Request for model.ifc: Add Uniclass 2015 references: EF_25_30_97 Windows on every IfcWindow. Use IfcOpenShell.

First a look at what the model holds.

```python
import ifcopenshell

model = ifcopenshell.open("model.ifc")
print(model.schema)
print("classifications:", [c.Name for c in model.by_type("IfcClassification")])
for ifc_class in ("IfcDoor", "IfcRoof", "IfcStair", "IfcWall", "IfcWindow"):
    print(ifc_class, len(model.by_type(ifc_class)))
```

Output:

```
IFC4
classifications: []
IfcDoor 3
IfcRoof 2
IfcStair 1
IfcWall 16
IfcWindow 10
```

```python
import ifcopenshell
import ifcopenshell.api.classification

model = ifcopenshell.open("model.ifc")

system = ifcopenshell.api.classification.add_classification(model, classification="Uniclass 2015")

codes = {
    "IfcWindow": ("EF_25_30_97", "Windows"),
}
for ifc_class, (code, name) in codes.items():
    products = model.by_type(ifc_class)
    ifcopenshell.api.classification.add_reference(
        model, products=products, classification=system, identification=code, name=name
    )
    print(code, len(products))

model.write("model_v2.ifc")
```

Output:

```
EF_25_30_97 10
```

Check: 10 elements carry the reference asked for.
